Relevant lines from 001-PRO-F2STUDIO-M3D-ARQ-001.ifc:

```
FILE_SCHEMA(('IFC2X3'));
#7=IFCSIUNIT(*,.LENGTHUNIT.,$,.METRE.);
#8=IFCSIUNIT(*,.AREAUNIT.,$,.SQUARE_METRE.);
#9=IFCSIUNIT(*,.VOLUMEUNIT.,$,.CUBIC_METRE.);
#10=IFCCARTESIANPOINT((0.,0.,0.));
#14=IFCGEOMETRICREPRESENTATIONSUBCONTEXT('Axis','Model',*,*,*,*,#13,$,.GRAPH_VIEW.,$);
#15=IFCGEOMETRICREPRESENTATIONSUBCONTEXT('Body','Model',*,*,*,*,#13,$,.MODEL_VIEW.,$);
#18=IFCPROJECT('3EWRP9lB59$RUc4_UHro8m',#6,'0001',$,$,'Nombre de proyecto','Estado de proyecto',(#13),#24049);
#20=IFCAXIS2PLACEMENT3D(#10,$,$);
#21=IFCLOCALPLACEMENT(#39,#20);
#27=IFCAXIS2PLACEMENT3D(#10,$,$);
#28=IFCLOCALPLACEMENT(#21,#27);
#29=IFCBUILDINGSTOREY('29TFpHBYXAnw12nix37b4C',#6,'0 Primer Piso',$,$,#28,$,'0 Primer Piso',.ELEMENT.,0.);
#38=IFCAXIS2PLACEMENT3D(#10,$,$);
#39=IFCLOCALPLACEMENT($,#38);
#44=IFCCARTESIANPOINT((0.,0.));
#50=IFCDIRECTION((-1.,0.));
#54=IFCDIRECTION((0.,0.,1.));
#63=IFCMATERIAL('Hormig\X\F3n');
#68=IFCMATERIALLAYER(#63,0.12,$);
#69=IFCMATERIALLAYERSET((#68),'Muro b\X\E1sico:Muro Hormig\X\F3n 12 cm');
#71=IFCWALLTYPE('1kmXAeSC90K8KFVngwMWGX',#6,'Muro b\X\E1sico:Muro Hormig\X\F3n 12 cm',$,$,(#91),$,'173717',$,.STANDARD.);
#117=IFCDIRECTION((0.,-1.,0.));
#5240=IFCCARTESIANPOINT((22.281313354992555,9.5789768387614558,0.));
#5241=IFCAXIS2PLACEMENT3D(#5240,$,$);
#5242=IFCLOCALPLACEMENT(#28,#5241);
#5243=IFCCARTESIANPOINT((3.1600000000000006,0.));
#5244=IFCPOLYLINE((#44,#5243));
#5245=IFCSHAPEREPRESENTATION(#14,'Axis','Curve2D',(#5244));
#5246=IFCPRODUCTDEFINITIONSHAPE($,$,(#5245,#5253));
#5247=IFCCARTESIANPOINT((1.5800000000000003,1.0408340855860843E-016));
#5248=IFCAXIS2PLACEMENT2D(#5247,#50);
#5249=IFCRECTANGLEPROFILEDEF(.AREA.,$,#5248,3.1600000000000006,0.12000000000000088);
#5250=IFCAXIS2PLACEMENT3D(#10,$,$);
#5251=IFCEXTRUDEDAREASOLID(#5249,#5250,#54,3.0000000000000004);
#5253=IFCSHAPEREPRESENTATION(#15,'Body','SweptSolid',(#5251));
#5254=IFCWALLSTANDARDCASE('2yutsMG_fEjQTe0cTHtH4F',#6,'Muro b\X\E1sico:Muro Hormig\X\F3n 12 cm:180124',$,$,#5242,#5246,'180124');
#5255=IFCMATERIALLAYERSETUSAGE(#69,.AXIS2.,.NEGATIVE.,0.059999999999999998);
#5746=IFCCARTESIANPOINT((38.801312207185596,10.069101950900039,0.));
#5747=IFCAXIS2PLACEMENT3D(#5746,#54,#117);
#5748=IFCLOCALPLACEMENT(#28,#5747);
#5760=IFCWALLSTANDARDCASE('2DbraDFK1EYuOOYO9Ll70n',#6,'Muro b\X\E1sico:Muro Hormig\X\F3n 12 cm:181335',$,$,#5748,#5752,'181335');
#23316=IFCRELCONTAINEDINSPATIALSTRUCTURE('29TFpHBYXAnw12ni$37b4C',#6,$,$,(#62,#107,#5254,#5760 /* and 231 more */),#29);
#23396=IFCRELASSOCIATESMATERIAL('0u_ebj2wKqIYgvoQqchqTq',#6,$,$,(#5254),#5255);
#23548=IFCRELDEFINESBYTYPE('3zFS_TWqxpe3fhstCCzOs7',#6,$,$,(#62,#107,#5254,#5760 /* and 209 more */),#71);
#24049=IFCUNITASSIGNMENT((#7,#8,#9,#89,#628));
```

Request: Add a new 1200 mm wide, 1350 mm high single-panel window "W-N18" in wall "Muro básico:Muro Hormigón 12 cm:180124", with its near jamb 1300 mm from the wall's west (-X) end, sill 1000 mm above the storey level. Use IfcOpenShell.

```python
import numpy as np
import ifcopenshell
import ifcopenshell.api.feature
import ifcopenshell.api.geometry
import ifcopenshell.api.root
import ifcopenshell.api.spatial
import ifcopenshell.api.type
import ifcopenshell.geom
import ifcopenshell.util.element
import ifcopenshell.util.placement
import ifcopenshell.util.representation
import ifcopenshell.util.shape
import ifcopenshell.util.unit

model = ifcopenshell.open("001-PRO-F2STUDIO-M3D-ARQ-001.ifc")
unit_scale = ifcopenshell.util.unit.calculate_unit_scale(model)
settings = ifcopenshell.geom.settings()


def volume(element):
    """Net volume in cubic metres, openings subtracted."""
    shape = ifcopenshell.geom.create_shape(settings, element)
    return ifcopenshell.util.shape.get_volume(shape.geometry)


wall = model.by_guid("2yutsMG_fEjQTe0cTHtH4F")
storey = ifcopenshell.util.element.get_container(wall, ifc_class="IfcBuildingStorey")
context = ifcopenshell.util.representation.get_context(model, "Model", "Body", "MODEL_VIEW")
before = volume(wall)

width, height, from_end, sill = 1.2, 1.35, 1.3, 1  # metres

# The wall runs along its own X axis, and the end named is its -X end.
wall_shape = ifcopenshell.geom.create_shape(settings, wall)
x, y, z = ifcopenshell.util.shape.get_vertices(wall_shape.geometry).T
start = x.min() + from_end
face, thickness = float(y.min()), float(y.max() - y.min())
wall_matrix = ifcopenshell.util.placement.get_local_placement(wall.ObjectPlacement)
level = ifcopenshell.util.placement.get_local_placement(storey.ObjectPlacement)[2, 3]


def in_wall(x, y):
    """Placement at x, y metres in the wall's axes, at sill height."""
    matrix = wall_matrix.copy()
    matrix[:, 3] = wall_matrix @ np.array([x / unit_scale, y / unit_scale, 0.0, 1.0])
    matrix[2, 3] = level + sill / unit_scale
    return matrix


# Opening: a box that overshoots both wall faces by 50 mm.
opening = ifcopenshell.api.root.create_entity(model, ifc_class="IfcOpeningElement")
box = ifcopenshell.api.geometry.add_wall_representation(
    model, context=context, length=width, height=height, thickness=thickness + 0.1
)
ifcopenshell.api.geometry.assign_representation(model, product=opening, representation=box)
ifcopenshell.api.geometry.edit_object_placement(model, product=opening, matrix=in_wall(start, face - 0.05), is_si=False)
ifcopenshell.api.feature.add_feature(model, feature=opening, element=wall)

window = ifcopenshell.api.root.create_entity(model, ifc_class="IfcWindow", name="W-N18")
window.OverallWidth, window.OverallHeight = width / unit_scale, height / unit_scale
body = ifcopenshell.api.geometry.add_window_representation(
    model,
    context=context,
    overall_width=window.OverallWidth,
    overall_height=window.OverallHeight,
    partition_type="SINGLE_PANEL",
)
ifcopenshell.api.geometry.assign_representation(model, product=window, representation=body)
ifcopenshell.api.spatial.assign_container(model, products=[window], relating_structure=storey)
fills = ifcopenshell.api.feature.add_filling(model, opening=opening, element=window)
fills.OwnerHistory = window.OwnerHistory  # required in IFC2X3

# IFC2X3 keeps the operation on the window style.
style = ifcopenshell.api.root.create_entity(model, ifc_class="IfcWindowStyle", name="W-N18")
style.OperationType, style.ConstructionType = "SINGLE_PANEL", "NOTDEFINED"
style.ParameterTakesPrecedence = style.Sizeable = False
ifcopenshell.api.type.assign_type(model, related_objects=[window], relating_type=style)

# Centre the window in the wall's thickness.
ifcopenshell.api.geometry.edit_object_placement(model, product=window, matrix=in_wall(start, face), is_si=False)
window_shape = ifcopenshell.geom.create_shape(settings, window)
depth = ifcopenshell.util.shape.get_vertices(window_shape.geometry)[:, 1]
offset = face + thickness / 2 - (depth.min() + depth.max()) / 2
ifcopenshell.api.geometry.edit_object_placement(model, product=window, matrix=in_wall(start, offset), is_si=False)

after = volume(wall)

print(f"wall volume {before:.3f} -> {after:.3f} m3")

model.write("001-PRO-F2STUDIO-M3D-ARQ-001_v2.ifc")
```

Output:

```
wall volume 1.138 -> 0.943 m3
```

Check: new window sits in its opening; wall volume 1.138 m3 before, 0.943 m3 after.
